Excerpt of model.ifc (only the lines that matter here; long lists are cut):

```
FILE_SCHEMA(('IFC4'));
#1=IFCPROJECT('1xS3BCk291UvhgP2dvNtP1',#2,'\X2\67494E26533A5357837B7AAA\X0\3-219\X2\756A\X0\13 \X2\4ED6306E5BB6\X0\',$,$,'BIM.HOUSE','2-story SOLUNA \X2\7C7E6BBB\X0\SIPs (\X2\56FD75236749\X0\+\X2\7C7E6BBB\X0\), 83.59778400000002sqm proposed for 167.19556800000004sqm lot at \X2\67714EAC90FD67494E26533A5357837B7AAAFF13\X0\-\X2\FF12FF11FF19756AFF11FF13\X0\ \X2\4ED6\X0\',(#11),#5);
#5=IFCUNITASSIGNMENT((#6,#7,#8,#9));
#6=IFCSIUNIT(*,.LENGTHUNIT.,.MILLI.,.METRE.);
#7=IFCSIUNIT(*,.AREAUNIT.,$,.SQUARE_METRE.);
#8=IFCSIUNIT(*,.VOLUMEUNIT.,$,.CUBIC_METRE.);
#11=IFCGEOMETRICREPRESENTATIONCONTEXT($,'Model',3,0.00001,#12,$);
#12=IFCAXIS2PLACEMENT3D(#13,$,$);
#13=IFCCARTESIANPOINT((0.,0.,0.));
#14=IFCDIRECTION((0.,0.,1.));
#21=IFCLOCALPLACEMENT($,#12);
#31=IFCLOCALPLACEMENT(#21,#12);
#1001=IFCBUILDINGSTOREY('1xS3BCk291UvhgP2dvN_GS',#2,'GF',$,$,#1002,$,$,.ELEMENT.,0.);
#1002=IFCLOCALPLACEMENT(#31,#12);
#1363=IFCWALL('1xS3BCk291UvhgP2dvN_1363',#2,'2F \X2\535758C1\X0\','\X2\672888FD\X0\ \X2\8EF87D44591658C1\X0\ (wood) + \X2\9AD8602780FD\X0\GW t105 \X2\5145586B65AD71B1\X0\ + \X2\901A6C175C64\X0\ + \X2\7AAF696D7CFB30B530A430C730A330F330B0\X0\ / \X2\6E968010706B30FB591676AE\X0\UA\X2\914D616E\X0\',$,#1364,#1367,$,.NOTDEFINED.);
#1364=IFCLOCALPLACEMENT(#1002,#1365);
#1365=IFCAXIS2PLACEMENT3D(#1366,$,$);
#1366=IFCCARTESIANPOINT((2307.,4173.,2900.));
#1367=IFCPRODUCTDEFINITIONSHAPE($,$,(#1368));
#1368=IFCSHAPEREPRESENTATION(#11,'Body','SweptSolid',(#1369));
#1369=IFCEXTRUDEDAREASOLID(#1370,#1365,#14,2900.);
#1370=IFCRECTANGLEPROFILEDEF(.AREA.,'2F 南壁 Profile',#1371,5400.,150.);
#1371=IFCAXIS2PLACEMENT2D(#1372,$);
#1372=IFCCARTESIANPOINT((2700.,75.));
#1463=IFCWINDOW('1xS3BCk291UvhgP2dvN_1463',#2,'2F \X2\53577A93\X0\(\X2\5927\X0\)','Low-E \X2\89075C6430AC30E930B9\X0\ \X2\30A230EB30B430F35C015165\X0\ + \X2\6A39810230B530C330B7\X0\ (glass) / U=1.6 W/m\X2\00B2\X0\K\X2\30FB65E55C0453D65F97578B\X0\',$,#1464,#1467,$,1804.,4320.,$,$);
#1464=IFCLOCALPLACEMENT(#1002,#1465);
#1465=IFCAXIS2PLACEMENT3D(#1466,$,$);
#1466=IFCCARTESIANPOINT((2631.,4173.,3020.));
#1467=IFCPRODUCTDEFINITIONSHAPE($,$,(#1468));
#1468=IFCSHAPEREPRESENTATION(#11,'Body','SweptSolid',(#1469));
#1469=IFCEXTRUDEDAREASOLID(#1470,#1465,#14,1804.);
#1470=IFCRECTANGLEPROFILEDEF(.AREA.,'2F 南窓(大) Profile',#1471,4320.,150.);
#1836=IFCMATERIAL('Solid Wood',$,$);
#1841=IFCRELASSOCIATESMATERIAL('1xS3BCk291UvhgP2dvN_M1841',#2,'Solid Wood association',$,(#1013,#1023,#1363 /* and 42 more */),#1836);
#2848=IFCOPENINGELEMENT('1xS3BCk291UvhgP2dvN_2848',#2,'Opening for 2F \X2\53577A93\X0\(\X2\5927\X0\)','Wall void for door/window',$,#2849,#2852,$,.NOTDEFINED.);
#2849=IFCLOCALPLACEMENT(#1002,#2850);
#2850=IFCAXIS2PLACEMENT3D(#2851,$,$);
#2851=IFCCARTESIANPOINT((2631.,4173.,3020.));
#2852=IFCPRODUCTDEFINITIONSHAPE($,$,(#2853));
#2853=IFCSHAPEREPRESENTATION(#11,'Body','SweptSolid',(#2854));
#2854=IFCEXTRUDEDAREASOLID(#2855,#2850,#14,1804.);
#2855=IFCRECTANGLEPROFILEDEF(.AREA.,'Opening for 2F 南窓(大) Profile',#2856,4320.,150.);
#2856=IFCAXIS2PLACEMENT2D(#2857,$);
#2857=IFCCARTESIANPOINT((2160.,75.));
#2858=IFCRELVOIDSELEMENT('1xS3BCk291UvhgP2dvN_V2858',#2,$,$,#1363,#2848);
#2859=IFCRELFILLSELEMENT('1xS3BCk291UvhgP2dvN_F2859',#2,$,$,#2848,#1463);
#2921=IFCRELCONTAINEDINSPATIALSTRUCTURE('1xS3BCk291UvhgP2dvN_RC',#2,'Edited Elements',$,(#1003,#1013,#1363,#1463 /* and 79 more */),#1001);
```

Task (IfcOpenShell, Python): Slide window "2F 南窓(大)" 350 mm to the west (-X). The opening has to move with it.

```python
import ifcopenshell
import ifcopenshell.api.geometry
import ifcopenshell.util.placement

model = ifcopenshell.open("model.ifc")

window = model.by_guid("1xS3BCk291UvhgP2dvN_1463")
opening = window.FillsVoids[0].RelatingOpeningElement
wall = opening.VoidsElements[0].RelatingBuildingElement

wall_matrix = ifcopenshell.util.placement.get_local_placement(wall.ObjectPlacement)
shift = wall_matrix[:3, 0] * -350.0
before = ifcopenshell.util.placement.get_local_placement(window.ObjectPlacement)[:3, 3].copy()

# The window is not placed relative to its opening, so move both.
for product in (opening, window):
    matrix = ifcopenshell.util.placement.get_local_placement(product.ObjectPlacement)
    matrix[:3, 3] += shift
    ifcopenshell.api.geometry.edit_object_placement(model, product=product, matrix=matrix, is_si=False)

after = ifcopenshell.util.placement.get_local_placement(window.ObjectPlacement)[:3, 3]
print("window moved by", (after - before).round(3) + 0.0)

model.write("model_rev.ifc")
```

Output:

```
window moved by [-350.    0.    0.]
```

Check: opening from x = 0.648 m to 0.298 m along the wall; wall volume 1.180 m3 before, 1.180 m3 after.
